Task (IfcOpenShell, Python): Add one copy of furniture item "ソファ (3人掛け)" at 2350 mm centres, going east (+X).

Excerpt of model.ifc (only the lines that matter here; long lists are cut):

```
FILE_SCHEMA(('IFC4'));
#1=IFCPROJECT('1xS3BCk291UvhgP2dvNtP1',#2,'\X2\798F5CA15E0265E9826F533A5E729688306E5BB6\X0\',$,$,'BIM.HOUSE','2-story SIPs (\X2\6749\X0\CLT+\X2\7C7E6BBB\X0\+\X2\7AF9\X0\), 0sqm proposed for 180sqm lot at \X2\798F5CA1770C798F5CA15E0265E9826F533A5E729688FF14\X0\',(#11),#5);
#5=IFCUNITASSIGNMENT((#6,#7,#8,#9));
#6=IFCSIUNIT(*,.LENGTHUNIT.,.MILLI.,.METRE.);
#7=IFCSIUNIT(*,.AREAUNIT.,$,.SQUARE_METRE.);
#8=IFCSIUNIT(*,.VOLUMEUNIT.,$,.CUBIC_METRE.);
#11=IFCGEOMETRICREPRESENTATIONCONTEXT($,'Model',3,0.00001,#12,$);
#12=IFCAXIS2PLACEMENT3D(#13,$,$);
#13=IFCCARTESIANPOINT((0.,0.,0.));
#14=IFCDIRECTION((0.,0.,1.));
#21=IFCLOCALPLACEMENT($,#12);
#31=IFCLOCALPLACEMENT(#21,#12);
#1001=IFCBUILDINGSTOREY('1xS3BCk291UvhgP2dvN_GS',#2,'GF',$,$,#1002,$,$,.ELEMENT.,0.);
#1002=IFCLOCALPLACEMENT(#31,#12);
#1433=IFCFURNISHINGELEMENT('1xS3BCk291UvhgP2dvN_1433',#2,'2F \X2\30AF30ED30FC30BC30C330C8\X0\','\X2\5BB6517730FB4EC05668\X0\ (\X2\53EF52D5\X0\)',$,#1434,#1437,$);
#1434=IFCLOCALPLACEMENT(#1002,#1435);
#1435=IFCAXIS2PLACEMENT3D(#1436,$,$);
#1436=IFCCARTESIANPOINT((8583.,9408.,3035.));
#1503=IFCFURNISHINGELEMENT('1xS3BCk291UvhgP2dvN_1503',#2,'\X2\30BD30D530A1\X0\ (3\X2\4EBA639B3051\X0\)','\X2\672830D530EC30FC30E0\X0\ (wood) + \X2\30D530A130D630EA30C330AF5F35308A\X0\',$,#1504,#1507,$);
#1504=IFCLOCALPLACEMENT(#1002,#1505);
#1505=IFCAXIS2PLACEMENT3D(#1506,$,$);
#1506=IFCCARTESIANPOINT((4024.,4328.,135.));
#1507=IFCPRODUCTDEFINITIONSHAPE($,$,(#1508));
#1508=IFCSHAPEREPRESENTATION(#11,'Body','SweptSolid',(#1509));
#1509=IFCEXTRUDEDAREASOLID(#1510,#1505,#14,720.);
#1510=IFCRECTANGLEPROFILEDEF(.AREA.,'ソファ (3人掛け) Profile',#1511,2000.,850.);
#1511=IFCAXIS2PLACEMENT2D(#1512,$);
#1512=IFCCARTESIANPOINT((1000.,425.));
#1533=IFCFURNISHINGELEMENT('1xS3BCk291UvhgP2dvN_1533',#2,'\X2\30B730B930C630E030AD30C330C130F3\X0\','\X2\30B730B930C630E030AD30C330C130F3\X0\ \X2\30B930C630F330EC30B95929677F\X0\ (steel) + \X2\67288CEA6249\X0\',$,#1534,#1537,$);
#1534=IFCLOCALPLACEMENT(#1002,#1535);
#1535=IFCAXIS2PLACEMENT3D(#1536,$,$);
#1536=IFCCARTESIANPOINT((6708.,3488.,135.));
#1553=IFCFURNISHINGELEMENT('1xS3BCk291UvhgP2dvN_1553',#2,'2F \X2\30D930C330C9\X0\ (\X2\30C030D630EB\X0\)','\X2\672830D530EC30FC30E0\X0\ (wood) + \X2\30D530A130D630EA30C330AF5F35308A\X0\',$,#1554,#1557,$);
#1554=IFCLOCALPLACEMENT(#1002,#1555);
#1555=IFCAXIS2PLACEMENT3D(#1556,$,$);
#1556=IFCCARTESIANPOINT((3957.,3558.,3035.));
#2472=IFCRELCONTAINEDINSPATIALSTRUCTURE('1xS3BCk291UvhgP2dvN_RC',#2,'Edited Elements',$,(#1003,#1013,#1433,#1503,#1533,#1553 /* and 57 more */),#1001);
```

```python
import numpy as np
import ifcopenshell
import ifcopenshell.api.geometry
import ifcopenshell.api.root
import ifcopenshell.util.element
import ifcopenshell.util.placement
import ifcopenshell.util.unit

model = ifcopenshell.open("model.ifc")
unit_scale = ifcopenshell.util.unit.calculate_unit_scale(model)


def reuse_history(source, copy):
    """copy_class also copies each property set's owner history, people and application; keep the originals."""
    for rel in copy.IsDefinedBy:
        if rel.is_a("IfcRelDefinesByProperties") and (history := rel.RelatingPropertyDefinition.OwnerHistory):
            rel.RelatingPropertyDefinition.OwnerHistory = source.OwnerHistory
            ifcopenshell.util.element.remove_deep2(model, history)


source = model.by_guid("1xS3BCk291UvhgP2dvN_1503")
base = ifcopenshell.util.placement.get_local_placement(source.ObjectPlacement)
step = np.array([1.0, 0.0, 0.0]) * 2.35 / unit_scale

for i in range(1, 2):
    copy = ifcopenshell.api.root.copy_class(model, product=source)
    copy.Representation = ifcopenshell.util.element.copy_deep(
        model, source.Representation, exclude=["IfcGeometricRepresentationContext", "IfcRepresentationMap"]
    )
    reuse_history(source, copy)
    matrix = base.copy()
    matrix[:3, 3] += i * step
    print("added at", matrix[:3, 3].round(3) + 0.0)
    ifcopenshell.api.geometry.edit_object_placement(model, product=copy, matrix=matrix, is_si=False)

model.write("model_rev.ifc")
```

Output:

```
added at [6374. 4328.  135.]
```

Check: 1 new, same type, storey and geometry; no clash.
